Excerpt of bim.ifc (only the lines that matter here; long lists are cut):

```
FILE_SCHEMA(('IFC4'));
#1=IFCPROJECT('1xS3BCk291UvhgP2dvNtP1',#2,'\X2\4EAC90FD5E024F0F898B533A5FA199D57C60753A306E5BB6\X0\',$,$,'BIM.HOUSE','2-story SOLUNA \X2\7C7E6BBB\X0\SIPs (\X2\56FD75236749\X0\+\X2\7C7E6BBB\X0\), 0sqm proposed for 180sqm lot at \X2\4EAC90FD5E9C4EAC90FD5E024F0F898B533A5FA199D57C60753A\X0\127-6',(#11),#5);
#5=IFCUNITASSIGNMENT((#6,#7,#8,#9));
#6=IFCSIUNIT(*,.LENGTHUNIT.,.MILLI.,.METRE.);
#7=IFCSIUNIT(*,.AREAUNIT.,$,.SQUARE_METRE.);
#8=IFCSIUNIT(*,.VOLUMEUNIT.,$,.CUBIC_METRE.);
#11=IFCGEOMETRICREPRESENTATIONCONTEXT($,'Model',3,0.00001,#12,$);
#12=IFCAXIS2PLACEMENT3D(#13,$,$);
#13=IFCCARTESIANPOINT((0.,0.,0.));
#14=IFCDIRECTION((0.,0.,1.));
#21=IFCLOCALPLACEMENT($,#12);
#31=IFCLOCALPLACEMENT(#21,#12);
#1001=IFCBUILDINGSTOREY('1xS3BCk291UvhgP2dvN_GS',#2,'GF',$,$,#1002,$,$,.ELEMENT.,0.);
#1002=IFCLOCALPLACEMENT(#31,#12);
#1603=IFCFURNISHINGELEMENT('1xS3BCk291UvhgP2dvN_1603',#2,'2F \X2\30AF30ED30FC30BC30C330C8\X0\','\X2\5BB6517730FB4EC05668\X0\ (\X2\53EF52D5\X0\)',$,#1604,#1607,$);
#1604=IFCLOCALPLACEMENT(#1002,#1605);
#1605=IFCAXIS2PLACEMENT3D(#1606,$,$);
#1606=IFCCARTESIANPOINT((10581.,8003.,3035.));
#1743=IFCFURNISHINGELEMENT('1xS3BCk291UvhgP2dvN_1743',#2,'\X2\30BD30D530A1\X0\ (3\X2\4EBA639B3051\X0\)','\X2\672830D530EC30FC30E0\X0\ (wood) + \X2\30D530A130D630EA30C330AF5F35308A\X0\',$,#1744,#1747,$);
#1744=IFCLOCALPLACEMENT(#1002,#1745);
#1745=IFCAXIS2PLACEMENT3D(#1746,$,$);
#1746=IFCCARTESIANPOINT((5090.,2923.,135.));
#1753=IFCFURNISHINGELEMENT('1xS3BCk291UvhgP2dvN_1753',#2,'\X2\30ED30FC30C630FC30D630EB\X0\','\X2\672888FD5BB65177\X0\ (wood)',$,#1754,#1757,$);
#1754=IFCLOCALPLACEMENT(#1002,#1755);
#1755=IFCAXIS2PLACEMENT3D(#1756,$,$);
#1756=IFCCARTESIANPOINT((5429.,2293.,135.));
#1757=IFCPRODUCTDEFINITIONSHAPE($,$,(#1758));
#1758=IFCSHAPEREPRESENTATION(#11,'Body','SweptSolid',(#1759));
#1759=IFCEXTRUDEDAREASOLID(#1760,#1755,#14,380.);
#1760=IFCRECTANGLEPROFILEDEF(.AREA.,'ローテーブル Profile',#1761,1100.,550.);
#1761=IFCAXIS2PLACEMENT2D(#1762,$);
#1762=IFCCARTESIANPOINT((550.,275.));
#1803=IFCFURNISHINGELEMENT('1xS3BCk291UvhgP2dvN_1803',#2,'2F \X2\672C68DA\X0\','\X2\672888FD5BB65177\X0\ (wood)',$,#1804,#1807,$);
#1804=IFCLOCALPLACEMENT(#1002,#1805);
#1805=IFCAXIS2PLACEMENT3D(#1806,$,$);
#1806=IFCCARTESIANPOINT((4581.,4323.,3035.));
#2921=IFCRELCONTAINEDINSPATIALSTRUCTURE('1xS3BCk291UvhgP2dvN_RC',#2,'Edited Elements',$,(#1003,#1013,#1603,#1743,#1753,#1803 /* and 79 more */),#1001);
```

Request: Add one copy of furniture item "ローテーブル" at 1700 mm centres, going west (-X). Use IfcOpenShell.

```python
import numpy as np
import ifcopenshell
import ifcopenshell.api.geometry
import ifcopenshell.api.root
import ifcopenshell.util.element
import ifcopenshell.util.placement

model = ifcopenshell.open("bim.ifc")


def reuse_history(source, copy):
    """copy_class also copies each property set's owner history, people and application; keep the originals."""
    for rel in copy.IsDefinedBy:
        if rel.is_a("IfcRelDefinesByProperties") and (history := rel.RelatingPropertyDefinition.OwnerHistory):
            rel.RelatingPropertyDefinition.OwnerHistory = source.OwnerHistory
            ifcopenshell.util.element.remove_deep2(model, history)


source = model.by_guid("1xS3BCk291UvhgP2dvN_1753")
base = ifcopenshell.util.placement.get_local_placement(source.ObjectPlacement)
step = np.array([-1.0, 0.0, 0.0]) * 1700.0

for i in range(1, 2):
    copy = ifcopenshell.api.root.copy_class(model, product=source)
    copy.Representation = ifcopenshell.util.element.copy_deep(
        model, source.Representation, exclude=["IfcGeometricRepresentationContext", "IfcRepresentationMap"]
    )
    reuse_history(source, copy)
    matrix = base.copy()
    matrix[:3, 3] += i * step
    print("added at", matrix[:3, 3].round(3) + 0.0)
    ifcopenshell.api.geometry.edit_object_placement(model, product=copy, matrix=matrix, is_si=False)

model.write("bim_edited.ifc")
```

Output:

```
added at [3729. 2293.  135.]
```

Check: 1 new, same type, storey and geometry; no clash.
